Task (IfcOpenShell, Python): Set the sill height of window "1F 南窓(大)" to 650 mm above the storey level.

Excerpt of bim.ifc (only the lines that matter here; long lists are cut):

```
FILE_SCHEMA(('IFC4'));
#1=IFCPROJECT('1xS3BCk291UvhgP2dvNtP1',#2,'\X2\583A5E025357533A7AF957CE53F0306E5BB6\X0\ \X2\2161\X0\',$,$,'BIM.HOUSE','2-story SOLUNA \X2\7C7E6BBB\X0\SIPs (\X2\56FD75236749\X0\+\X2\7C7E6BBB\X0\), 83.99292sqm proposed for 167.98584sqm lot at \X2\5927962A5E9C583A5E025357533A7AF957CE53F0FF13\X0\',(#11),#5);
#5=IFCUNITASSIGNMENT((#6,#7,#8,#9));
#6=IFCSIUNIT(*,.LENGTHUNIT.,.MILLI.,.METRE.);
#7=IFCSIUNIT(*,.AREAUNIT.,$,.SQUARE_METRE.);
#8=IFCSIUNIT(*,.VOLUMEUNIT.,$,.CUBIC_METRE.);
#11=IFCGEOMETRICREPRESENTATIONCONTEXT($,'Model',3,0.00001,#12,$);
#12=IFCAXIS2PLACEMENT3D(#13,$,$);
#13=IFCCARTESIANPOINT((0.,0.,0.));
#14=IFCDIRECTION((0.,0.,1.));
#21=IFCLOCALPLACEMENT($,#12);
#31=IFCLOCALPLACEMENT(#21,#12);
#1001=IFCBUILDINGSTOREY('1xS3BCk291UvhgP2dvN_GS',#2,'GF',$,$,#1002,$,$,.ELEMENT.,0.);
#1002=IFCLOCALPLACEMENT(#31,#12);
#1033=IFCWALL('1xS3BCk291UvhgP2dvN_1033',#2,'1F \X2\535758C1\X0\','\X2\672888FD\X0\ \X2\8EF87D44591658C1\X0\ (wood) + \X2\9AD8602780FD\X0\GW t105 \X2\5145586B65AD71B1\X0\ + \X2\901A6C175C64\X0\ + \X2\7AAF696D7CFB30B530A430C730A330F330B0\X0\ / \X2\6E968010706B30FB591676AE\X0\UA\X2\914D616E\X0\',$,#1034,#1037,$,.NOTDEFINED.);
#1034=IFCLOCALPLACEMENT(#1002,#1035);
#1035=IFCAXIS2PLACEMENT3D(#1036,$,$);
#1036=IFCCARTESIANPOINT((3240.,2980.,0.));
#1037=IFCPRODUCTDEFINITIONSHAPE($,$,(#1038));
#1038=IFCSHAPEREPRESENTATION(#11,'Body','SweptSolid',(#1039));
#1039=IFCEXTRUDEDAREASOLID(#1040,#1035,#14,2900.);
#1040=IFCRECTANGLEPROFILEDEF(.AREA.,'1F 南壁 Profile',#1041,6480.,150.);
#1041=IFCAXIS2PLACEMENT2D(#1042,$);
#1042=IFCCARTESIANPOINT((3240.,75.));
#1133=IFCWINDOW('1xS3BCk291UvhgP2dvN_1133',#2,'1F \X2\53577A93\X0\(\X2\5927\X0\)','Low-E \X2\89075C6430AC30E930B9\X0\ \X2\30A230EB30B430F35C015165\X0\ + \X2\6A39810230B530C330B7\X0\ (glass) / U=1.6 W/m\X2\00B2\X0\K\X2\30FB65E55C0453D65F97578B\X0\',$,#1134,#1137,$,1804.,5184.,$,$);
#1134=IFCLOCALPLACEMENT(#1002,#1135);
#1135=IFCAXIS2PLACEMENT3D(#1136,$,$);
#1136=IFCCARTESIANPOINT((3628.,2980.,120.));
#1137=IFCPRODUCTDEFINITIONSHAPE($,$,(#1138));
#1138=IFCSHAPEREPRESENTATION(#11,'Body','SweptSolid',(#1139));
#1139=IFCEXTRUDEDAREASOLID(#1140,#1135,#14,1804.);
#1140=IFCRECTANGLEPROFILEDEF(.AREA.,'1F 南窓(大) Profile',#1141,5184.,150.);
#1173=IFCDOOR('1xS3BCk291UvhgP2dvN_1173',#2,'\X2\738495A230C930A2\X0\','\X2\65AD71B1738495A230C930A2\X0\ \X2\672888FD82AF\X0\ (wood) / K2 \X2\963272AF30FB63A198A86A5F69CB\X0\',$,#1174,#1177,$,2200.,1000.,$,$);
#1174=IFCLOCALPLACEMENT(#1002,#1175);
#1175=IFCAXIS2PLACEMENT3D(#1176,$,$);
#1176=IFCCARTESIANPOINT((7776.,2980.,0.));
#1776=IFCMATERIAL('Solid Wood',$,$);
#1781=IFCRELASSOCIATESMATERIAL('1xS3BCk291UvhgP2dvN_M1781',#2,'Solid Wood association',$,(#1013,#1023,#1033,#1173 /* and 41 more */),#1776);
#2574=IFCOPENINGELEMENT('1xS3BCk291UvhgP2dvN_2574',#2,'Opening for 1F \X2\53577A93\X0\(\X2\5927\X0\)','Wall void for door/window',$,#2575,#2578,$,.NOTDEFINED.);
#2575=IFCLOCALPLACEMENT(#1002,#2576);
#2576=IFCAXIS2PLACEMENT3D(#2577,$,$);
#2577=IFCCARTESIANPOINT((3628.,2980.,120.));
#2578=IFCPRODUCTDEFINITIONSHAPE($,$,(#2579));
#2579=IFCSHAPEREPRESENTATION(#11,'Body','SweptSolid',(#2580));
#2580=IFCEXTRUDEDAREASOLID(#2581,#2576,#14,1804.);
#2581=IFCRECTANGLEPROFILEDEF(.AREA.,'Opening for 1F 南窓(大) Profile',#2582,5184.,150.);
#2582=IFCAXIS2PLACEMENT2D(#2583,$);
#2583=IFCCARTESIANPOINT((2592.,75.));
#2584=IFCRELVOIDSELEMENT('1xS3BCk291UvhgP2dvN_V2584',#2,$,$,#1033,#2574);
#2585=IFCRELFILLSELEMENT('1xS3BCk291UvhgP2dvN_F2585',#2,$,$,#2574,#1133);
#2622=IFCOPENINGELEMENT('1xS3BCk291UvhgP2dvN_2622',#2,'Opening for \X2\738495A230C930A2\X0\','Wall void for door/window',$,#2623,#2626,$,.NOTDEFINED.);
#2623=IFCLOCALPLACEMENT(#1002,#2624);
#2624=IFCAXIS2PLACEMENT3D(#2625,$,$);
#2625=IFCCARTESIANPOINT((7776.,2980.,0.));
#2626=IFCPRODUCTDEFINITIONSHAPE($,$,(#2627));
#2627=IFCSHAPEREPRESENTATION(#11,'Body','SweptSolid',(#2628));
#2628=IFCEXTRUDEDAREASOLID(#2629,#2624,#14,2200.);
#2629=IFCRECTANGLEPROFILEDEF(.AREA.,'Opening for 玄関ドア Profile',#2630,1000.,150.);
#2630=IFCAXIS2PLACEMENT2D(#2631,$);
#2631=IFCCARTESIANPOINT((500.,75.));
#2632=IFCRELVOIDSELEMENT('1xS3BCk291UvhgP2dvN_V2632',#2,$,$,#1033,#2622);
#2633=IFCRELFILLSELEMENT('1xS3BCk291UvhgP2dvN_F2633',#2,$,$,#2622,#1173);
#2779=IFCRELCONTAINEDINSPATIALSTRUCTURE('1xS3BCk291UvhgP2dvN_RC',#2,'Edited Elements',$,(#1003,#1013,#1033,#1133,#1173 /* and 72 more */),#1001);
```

```python
import numpy as np
import ifcopenshell
import ifcopenshell.api.geometry
import ifcopenshell.geom
import ifcopenshell.util.element
import ifcopenshell.util.placement
import ifcopenshell.util.shape
import ifcopenshell.util.unit

model = ifcopenshell.open("bim.ifc")
unit_scale = ifcopenshell.util.unit.calculate_unit_scale(model)

window = model.by_guid("1xS3BCk291UvhgP2dvN_1133")
opening = window.FillsVoids[0].RelatingOpeningElement
storey = ifcopenshell.util.element.get_container(window, ifc_class="IfcBuildingStorey")
level = ifcopenshell.util.placement.get_local_placement(storey.ObjectPlacement)[2, 3]

# The opening's origin need not be at the sill, so measure its lowest point.
shape = ifcopenshell.geom.create_shape(ifcopenshell.geom.settings(), opening)
bottom = ifcopenshell.util.shape.get_shape_bottom_elevation(shape, shape.geometry) / unit_scale
dz = level + 0.65 / unit_scale - bottom

shift = np.array([0.0, 0.0, dz])
# The window is not placed relative to its opening, so move both.
for product in (opening, window):
    matrix = ifcopenshell.util.placement.get_local_placement(product.ObjectPlacement)
    matrix[:3, 3] += shift
    ifcopenshell.api.geometry.edit_object_placement(model, product=product, matrix=matrix, is_si=False)

print(f"moved by {dz * unit_scale:+.3f} m")

model.write("bim-out.ifc")
```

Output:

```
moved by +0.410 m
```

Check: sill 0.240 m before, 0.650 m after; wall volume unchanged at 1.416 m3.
